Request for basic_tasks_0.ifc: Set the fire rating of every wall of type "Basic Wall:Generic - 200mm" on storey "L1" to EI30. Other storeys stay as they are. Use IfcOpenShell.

First a look at what the model holds.

```python
import ifcopenshell
import ifcopenshell.util.element

model = ifcopenshell.open("basic_tasks_0.ifc")
print(model.schema)
storey = next(s for s in model.by_type("IfcBuildingStorey") if s.Name == "L1")
walls = [e for e in ifcopenshell.util.element.get_decomposition(storey) if e.is_a("IfcWall")]
seen = {}
for e in walls:
    element_type = ifcopenshell.util.element.get_type(e)
    key = (element_type.Name if element_type != e and element_type else None, ifcopenshell.util.element.get_pset(e, "Pset_WallCommon", "FireRating"))
    seen[key] = seen.get(key, 0) + 1
for (name, value), count in sorted(seen.items(), key=str):
    print(count, "x", name, "|", value)
```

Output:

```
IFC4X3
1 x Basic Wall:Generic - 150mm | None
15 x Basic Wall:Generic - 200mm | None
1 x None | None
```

```python
import ifcopenshell
import ifcopenshell.api.pset
import ifcopenshell.util.element

model = ifcopenshell.open("basic_tasks_0.ifc")

storey = next(s for s in model.by_type("IfcBuildingStorey") if s.Name == "L1")
walls = [e for e in ifcopenshell.util.element.get_decomposition(storey) if e.is_a("IfcWall")]

count = 0
for e in walls:
    element_type = ifcopenshell.util.element.get_type(e)
    if element_type in (None, e) or element_type.Name != "Basic Wall:Generic - 200mm":
        continue
    # add_pset returns the element's existing set when there is one.
    pset = ifcopenshell.api.pset.add_pset(model, product=e, name="Pset_WallCommon")
    ifcopenshell.api.pset.edit_pset(model, pset=pset, properties={"FireRating": "EI30"})
    count += 1

print(count, "walls updated")

model.write("basic_tasks_0_edited.ifc")
```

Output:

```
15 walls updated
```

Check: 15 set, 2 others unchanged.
